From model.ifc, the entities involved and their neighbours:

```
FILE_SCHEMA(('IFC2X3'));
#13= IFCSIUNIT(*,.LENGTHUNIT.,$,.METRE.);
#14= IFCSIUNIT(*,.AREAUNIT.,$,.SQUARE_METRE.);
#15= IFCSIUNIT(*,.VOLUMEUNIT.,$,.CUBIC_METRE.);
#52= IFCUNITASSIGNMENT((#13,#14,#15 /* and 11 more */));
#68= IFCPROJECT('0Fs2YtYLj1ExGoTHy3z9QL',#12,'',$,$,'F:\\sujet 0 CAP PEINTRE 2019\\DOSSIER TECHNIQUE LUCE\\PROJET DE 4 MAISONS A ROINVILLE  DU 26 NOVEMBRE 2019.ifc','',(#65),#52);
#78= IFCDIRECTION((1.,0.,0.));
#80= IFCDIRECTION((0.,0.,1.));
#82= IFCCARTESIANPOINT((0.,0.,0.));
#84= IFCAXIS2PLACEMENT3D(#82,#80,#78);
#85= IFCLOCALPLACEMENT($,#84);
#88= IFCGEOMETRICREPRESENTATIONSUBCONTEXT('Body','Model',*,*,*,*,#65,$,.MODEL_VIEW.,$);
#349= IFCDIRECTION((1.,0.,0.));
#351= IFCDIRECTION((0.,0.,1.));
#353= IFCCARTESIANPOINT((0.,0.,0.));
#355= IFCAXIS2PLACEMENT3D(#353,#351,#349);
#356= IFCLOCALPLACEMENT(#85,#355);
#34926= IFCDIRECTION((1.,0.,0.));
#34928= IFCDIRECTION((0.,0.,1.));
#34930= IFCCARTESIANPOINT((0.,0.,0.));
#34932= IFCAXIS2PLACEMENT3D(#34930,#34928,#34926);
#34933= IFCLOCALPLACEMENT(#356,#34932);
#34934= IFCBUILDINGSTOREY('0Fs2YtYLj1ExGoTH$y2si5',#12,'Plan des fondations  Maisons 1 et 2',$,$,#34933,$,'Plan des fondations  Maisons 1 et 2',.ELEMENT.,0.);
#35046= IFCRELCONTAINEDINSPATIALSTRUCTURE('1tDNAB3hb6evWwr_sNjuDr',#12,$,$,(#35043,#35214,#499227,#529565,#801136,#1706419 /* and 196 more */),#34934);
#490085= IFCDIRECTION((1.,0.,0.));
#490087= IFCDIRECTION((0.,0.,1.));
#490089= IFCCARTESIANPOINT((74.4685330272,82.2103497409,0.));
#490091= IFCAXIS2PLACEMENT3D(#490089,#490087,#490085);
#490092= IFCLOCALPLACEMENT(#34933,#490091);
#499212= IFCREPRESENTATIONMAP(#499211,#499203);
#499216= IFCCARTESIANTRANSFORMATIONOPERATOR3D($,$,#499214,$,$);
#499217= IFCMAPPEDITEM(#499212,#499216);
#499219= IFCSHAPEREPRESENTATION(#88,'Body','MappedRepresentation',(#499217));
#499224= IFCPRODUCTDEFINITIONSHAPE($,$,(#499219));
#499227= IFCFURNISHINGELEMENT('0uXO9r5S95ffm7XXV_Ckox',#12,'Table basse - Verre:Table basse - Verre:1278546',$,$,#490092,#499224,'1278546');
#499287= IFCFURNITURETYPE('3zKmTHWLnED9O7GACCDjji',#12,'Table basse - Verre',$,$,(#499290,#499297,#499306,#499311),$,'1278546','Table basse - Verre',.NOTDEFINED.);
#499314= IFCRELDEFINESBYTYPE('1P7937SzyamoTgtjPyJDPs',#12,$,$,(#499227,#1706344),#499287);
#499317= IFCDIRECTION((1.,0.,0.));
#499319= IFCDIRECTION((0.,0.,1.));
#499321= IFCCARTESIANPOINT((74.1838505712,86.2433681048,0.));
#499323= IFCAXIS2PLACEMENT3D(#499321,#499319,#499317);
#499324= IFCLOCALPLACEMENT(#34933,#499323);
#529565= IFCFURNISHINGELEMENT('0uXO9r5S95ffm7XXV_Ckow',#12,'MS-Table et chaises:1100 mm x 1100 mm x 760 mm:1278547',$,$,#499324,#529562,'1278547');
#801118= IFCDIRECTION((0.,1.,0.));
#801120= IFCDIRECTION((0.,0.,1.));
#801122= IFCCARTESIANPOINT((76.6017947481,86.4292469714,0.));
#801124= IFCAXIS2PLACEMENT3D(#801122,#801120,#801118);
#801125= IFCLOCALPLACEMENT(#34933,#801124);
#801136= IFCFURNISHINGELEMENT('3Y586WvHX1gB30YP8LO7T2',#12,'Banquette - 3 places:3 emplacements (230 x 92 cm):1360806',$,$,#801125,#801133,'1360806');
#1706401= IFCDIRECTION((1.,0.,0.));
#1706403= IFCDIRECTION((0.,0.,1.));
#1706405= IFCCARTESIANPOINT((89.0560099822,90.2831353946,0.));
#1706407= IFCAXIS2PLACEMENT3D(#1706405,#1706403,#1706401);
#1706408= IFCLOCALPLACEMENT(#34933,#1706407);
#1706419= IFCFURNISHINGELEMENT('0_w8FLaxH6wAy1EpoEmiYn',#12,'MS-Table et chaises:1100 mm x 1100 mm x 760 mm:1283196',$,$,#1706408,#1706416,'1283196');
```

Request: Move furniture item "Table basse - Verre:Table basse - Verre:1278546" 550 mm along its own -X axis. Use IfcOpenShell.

```python
import ifcopenshell
import ifcopenshell.api.geometry
import ifcopenshell.util.placement
import ifcopenshell.util.unit

model = ifcopenshell.open("model.ifc")
unit_scale = ifcopenshell.util.unit.calculate_unit_scale(model)

item = model.by_id(499227)
matrix = ifcopenshell.util.placement.get_local_placement(item.ObjectPlacement)
matrix[:3, 3] -= matrix[:3, 0] * 0.55 / unit_scale
ifcopenshell.api.geometry.edit_object_placement(model, product=item, matrix=matrix, is_si=False)

print(ifcopenshell.util.placement.get_local_placement(item.ObjectPlacement).round(3) + 0.0)

model.write("model_updated.ifc")
```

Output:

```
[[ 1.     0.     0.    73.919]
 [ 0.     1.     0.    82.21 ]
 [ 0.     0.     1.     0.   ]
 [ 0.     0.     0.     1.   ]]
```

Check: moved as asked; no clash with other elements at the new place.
